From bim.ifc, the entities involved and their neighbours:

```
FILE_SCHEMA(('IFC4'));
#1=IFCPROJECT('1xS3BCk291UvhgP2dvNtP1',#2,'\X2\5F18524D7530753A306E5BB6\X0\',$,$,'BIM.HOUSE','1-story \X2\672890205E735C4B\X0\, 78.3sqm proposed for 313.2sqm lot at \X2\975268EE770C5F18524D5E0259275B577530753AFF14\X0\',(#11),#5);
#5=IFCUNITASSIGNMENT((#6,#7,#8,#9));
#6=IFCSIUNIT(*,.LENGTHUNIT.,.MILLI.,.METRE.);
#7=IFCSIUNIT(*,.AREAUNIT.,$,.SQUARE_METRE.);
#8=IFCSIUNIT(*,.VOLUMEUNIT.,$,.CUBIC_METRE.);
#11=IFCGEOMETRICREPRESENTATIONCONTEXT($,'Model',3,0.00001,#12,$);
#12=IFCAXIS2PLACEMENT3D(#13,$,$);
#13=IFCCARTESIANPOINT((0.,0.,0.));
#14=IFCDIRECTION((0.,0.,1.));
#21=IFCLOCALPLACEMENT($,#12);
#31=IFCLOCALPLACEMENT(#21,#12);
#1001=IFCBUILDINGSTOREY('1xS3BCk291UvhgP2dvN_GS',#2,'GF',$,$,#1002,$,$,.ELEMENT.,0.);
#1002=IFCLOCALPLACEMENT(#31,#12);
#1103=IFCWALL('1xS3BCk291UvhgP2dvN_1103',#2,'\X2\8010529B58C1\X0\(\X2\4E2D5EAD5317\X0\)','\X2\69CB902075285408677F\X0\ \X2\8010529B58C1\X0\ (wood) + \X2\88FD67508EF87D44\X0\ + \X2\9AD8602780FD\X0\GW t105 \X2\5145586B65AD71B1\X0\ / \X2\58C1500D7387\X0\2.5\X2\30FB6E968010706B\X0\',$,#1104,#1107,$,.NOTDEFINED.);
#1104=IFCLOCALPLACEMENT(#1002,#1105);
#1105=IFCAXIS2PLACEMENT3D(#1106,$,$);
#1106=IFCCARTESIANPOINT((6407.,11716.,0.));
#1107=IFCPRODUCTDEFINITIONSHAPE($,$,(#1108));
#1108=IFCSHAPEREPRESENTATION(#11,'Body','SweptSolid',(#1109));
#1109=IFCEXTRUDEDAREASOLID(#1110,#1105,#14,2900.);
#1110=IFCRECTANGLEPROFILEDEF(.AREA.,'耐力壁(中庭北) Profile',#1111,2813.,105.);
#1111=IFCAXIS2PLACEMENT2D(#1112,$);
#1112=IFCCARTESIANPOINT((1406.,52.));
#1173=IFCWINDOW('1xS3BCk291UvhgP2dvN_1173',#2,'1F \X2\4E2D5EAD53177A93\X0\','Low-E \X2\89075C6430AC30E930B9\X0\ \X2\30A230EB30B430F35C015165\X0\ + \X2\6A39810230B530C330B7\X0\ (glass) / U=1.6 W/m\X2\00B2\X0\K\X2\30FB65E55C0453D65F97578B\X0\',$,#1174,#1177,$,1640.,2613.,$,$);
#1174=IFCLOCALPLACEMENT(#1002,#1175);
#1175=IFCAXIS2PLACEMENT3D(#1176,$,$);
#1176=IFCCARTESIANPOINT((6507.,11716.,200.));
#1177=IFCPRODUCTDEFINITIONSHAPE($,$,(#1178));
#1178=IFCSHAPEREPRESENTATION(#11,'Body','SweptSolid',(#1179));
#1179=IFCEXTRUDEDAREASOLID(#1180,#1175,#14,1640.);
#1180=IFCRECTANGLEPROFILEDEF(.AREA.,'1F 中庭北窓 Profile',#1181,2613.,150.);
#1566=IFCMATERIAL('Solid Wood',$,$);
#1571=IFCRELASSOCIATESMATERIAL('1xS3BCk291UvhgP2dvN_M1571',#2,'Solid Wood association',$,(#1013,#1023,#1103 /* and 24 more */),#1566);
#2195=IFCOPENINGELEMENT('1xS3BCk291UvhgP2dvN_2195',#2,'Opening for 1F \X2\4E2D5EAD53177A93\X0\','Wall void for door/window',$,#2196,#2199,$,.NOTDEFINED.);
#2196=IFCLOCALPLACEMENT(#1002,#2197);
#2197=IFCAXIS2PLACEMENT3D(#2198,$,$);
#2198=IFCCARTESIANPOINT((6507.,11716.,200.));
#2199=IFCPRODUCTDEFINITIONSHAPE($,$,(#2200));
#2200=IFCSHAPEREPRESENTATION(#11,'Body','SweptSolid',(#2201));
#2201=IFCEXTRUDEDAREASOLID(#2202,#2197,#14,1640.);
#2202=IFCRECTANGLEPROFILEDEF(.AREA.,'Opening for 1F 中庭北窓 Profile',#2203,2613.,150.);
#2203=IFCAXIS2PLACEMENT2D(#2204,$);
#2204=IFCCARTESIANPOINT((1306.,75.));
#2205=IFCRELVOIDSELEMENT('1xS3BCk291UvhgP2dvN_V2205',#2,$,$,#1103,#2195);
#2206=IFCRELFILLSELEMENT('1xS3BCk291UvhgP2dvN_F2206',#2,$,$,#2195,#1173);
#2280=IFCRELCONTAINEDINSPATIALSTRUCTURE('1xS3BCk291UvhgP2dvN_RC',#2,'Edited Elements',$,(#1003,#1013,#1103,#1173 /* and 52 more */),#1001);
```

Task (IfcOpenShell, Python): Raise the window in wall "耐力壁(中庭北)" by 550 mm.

```python
import numpy as np
import ifcopenshell
import ifcopenshell.api.geometry
import ifcopenshell.util.placement
import ifcopenshell.util.unit

model = ifcopenshell.open("bim.ifc")
unit_scale = ifcopenshell.util.unit.calculate_unit_scale(model)

window = model.by_guid("1xS3BCk291UvhgP2dvN_1173")
opening = window.FillsVoids[0].RelatingOpeningElement
dz = 0.55 / unit_scale

shift = np.array([0.0, 0.0, dz])
# The window is not placed relative to its opening, so move both.
for product in (opening, window):
    matrix = ifcopenshell.util.placement.get_local_placement(product.ObjectPlacement)
    matrix[:3, 3] += shift
    ifcopenshell.api.geometry.edit_object_placement(model, product=product, matrix=matrix, is_si=False)

print(f"moved by {dz * unit_scale:+.3f} m")

model.write("bim_edited.ifc")
```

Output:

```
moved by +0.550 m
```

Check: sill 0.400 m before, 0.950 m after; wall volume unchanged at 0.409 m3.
